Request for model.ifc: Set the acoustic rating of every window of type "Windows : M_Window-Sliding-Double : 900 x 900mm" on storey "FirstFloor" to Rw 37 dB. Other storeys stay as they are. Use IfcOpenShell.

First a look at what the model holds.

```python
import ifcopenshell
import ifcopenshell.util.element

model = ifcopenshell.open("model.ifc")
print(model.schema)
storey = next(s for s in model.by_type("IfcBuildingStorey") if s.Name == "FirstFloor")
windows = [e for e in ifcopenshell.util.element.get_decomposition(storey) if e.is_a("IfcWindow")]
seen = {}
for e in windows:
    element_type = ifcopenshell.util.element.get_type(e)
    key = (element_type.Name if element_type != e and element_type else None, ifcopenshell.util.element.get_pset(e, "Pset_WindowCommon", "AcousticRating"))
    seen[key] = seen.get(key, 0) + 1
for (name, value), count in sorted(seen.items(), key=str):
    print(count, "x", name, "|", value)
```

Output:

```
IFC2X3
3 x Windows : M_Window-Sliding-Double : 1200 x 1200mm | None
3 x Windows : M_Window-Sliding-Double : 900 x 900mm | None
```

```python
import ifcopenshell
import ifcopenshell.api.pset
import ifcopenshell.util.element

model = ifcopenshell.open("model.ifc")

storey = next(s for s in model.by_type("IfcBuildingStorey") if s.Name == "FirstFloor")
windows = [e for e in ifcopenshell.util.element.get_decomposition(storey) if e.is_a("IfcWindow")]

count = 0
for e in windows:
    element_type = ifcopenshell.util.element.get_type(e)
    if element_type in (None, e) or element_type.Name != "Windows : M_Window-Sliding-Double : 900 x 900mm":
        continue
    # add_pset returns the element's existing set when there is one.
    pset = ifcopenshell.api.pset.add_pset(model, product=e, name="Pset_WindowCommon")
    ifcopenshell.api.pset.edit_pset(model, pset=pset, properties={"AcousticRating": "Rw 37 dB"})
    count += 1

print(count, "windows updated")

model.write("model_edited.ifc")
```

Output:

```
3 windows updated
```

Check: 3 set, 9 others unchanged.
